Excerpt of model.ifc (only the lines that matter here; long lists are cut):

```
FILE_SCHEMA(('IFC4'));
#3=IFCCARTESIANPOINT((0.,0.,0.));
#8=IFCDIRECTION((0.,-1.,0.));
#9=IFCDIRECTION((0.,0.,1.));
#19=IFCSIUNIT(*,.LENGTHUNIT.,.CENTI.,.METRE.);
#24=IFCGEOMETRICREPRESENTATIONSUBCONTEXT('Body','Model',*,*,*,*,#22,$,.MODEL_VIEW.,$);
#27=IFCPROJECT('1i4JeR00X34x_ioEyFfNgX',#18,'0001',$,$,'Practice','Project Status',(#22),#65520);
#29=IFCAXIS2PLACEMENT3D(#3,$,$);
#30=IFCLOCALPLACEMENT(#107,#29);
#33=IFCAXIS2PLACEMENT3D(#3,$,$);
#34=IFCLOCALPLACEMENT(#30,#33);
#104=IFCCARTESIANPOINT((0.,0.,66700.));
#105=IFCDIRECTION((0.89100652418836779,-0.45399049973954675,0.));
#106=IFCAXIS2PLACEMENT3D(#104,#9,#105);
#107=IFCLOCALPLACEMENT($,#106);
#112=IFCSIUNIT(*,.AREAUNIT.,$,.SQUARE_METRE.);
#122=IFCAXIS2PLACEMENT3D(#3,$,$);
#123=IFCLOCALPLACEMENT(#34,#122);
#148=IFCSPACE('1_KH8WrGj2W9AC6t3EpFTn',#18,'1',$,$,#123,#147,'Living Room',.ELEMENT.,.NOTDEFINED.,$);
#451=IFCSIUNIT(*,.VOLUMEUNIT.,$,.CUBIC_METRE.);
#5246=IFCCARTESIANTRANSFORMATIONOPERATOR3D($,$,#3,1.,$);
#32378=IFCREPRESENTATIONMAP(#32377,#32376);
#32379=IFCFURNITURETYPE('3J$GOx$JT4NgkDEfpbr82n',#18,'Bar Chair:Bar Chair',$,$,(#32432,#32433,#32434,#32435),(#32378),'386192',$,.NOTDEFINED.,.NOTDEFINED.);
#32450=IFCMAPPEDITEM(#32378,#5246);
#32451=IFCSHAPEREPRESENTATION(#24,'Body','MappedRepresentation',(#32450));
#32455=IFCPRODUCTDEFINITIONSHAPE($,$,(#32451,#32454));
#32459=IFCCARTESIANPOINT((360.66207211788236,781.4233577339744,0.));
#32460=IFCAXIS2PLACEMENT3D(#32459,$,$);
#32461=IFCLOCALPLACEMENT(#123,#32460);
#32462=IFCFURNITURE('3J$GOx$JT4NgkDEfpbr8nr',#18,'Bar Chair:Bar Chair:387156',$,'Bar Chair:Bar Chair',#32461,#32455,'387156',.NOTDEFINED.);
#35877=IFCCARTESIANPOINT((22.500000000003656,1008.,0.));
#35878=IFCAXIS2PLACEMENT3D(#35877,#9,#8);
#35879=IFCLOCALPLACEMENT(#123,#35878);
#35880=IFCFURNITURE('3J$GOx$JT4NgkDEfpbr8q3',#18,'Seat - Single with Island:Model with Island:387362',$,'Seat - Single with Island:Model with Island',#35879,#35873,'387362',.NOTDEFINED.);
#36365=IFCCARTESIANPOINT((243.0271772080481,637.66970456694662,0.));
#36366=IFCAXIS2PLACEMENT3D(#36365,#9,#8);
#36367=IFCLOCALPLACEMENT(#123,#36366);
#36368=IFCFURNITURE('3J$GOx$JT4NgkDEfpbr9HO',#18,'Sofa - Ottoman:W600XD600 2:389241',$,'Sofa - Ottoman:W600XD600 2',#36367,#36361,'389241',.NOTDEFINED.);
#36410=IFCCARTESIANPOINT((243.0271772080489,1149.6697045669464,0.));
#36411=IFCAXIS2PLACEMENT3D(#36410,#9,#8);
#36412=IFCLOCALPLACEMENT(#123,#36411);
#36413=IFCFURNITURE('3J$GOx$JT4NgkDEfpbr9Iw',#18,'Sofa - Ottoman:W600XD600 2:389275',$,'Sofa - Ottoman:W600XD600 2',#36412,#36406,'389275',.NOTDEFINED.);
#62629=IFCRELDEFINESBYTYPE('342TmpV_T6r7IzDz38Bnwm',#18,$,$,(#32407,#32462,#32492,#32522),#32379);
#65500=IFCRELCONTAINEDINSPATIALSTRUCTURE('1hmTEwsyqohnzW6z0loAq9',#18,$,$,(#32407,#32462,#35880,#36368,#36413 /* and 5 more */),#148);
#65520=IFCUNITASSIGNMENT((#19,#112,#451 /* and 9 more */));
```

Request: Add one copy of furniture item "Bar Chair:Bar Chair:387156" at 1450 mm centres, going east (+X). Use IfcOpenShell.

```python
import numpy as np
import ifcopenshell
import ifcopenshell.api.geometry
import ifcopenshell.api.root
import ifcopenshell.util.element
import ifcopenshell.util.placement
import ifcopenshell.util.unit

model = ifcopenshell.open("model.ifc")
unit_scale = ifcopenshell.util.unit.calculate_unit_scale(model)


def reuse_history(source, copy):
    """copy_class also copies each property set's owner history, people and application; keep the originals."""
    for rel in copy.IsDefinedBy:
        if rel.is_a("IfcRelDefinesByProperties") and (history := rel.RelatingPropertyDefinition.OwnerHistory):
            rel.RelatingPropertyDefinition.OwnerHistory = source.OwnerHistory
            ifcopenshell.util.element.remove_deep2(model, history)


source = model.by_guid("3J$GOx$JT4NgkDEfpbr8nr")
base = ifcopenshell.util.placement.get_local_placement(source.ObjectPlacement)
step = np.array([1.0, 0.0, 0.0]) * 1.45 / unit_scale

for i in range(1, 2):
    copy = ifcopenshell.api.root.copy_class(model, product=source)
    copy.Representation = ifcopenshell.util.element.copy_deep(
        model, source.Representation, exclude=["IfcGeometricRepresentationContext", "IfcRepresentationMap"]
    )
    copy.Name = "Bar Chair:Bar Chair"
    copy.Tag = None
    reuse_history(source, copy)
    matrix = base.copy()
    matrix[:3, 3] += i * step
    print("added at", matrix[:3, 3].round(3) + 0.0)
    ifcopenshell.api.geometry.edit_object_placement(model, product=copy, matrix=matrix, is_si=False)

model.write("model-out.ifc")
```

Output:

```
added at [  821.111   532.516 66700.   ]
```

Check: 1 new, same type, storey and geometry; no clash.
